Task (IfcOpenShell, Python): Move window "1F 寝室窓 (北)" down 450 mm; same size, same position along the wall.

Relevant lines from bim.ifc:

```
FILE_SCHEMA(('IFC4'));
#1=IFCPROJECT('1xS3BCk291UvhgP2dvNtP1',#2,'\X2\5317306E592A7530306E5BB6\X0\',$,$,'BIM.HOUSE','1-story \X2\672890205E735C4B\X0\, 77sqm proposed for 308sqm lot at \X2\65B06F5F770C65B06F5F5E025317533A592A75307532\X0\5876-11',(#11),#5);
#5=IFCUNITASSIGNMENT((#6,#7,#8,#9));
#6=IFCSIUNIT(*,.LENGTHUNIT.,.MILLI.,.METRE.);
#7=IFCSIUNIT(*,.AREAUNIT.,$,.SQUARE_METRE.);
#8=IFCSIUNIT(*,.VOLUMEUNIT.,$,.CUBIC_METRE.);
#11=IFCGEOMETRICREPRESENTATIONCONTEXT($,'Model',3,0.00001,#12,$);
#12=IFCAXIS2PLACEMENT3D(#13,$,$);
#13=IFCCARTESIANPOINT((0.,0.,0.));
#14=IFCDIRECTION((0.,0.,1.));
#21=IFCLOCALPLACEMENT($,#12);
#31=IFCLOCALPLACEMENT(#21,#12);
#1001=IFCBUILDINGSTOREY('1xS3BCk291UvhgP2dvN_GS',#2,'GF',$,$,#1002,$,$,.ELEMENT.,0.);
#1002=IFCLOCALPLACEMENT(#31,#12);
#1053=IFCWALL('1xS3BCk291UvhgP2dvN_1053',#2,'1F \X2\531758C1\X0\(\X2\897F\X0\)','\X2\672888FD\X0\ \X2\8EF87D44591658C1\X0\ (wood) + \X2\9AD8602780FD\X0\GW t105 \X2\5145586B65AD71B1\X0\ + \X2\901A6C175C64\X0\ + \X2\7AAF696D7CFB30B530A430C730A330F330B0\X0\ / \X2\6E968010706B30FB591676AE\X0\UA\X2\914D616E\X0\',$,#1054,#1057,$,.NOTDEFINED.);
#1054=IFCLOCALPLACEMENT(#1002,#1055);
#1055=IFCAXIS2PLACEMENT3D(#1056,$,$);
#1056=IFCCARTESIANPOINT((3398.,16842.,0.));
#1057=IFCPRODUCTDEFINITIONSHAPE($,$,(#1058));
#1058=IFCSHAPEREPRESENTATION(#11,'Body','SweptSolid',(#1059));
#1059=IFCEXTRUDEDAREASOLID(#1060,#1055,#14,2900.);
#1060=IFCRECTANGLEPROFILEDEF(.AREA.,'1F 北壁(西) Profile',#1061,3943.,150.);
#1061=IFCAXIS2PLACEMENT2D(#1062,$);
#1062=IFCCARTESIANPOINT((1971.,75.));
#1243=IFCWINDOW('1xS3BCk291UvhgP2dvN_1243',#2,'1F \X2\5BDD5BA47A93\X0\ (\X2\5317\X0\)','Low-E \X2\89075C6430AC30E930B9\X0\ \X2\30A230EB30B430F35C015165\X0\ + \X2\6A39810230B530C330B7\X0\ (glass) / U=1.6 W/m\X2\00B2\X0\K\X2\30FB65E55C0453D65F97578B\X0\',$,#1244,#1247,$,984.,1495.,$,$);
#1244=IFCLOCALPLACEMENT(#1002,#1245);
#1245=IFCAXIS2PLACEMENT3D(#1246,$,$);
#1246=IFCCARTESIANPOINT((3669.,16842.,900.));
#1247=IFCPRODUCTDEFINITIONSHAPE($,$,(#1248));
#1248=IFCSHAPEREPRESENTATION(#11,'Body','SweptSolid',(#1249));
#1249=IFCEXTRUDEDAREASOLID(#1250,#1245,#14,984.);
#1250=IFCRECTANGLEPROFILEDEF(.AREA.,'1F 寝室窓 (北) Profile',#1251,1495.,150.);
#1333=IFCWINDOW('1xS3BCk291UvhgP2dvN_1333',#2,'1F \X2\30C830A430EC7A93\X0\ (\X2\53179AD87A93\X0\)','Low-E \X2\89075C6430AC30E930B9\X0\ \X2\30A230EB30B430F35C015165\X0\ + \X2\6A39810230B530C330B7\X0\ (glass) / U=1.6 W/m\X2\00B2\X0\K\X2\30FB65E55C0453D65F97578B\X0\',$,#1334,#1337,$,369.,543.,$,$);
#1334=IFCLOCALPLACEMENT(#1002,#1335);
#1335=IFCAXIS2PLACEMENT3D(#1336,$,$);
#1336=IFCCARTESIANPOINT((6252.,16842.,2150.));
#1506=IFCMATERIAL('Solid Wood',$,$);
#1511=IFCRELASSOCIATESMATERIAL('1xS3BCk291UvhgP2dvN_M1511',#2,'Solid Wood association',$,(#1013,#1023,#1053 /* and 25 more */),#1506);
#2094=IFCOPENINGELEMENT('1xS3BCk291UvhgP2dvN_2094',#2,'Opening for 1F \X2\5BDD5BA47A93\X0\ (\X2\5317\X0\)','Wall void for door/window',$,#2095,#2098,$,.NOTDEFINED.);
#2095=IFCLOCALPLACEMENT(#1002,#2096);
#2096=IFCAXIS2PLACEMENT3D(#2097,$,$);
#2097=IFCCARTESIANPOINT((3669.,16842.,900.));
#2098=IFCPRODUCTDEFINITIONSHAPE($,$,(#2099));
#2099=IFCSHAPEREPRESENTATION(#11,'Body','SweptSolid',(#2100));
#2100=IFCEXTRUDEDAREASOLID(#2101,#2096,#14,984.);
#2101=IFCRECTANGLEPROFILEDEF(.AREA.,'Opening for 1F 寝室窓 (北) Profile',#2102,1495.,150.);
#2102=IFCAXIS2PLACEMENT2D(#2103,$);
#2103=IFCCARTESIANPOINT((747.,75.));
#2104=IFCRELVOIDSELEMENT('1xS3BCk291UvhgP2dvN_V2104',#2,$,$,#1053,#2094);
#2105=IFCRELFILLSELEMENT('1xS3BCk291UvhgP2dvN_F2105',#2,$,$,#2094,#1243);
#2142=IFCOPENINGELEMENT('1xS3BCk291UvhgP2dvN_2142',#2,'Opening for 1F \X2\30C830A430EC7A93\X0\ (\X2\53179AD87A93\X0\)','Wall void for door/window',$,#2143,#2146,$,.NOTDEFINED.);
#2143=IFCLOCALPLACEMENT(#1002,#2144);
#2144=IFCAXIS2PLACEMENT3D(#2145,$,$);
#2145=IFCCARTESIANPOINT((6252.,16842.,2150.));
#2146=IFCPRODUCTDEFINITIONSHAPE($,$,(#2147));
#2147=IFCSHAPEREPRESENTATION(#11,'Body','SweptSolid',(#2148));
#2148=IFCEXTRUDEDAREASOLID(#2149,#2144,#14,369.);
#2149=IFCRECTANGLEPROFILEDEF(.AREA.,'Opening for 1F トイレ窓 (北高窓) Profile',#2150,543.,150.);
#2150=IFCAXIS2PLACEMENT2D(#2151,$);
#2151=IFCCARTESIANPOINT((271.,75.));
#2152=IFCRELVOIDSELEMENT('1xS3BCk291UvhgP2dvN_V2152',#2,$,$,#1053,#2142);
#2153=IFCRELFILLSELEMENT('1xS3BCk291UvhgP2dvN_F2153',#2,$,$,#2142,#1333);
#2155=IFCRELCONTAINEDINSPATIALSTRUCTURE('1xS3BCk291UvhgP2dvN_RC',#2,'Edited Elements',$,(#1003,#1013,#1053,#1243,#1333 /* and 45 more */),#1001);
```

```python
import numpy as np
import ifcopenshell
import ifcopenshell.api.geometry
import ifcopenshell.util.placement
import ifcopenshell.util.unit

model = ifcopenshell.open("bim.ifc")
unit_scale = ifcopenshell.util.unit.calculate_unit_scale(model)

window = model.by_guid("1xS3BCk291UvhgP2dvN_1243")
opening = window.FillsVoids[0].RelatingOpeningElement
dz = -450.0

shift = np.array([0.0, 0.0, dz])
# The window is not placed relative to its opening, so move both.
for product in (opening, window):
    matrix = ifcopenshell.util.placement.get_local_placement(product.ObjectPlacement)
    matrix[:3, 3] += shift
    ifcopenshell.api.geometry.edit_object_placement(model, product=product, matrix=matrix, is_si=False)

print(f"moved by {dz * unit_scale:+.3f} m")

model.write("bim_rev.ifc")
```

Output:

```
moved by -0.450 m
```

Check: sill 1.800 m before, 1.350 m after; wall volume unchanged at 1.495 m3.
